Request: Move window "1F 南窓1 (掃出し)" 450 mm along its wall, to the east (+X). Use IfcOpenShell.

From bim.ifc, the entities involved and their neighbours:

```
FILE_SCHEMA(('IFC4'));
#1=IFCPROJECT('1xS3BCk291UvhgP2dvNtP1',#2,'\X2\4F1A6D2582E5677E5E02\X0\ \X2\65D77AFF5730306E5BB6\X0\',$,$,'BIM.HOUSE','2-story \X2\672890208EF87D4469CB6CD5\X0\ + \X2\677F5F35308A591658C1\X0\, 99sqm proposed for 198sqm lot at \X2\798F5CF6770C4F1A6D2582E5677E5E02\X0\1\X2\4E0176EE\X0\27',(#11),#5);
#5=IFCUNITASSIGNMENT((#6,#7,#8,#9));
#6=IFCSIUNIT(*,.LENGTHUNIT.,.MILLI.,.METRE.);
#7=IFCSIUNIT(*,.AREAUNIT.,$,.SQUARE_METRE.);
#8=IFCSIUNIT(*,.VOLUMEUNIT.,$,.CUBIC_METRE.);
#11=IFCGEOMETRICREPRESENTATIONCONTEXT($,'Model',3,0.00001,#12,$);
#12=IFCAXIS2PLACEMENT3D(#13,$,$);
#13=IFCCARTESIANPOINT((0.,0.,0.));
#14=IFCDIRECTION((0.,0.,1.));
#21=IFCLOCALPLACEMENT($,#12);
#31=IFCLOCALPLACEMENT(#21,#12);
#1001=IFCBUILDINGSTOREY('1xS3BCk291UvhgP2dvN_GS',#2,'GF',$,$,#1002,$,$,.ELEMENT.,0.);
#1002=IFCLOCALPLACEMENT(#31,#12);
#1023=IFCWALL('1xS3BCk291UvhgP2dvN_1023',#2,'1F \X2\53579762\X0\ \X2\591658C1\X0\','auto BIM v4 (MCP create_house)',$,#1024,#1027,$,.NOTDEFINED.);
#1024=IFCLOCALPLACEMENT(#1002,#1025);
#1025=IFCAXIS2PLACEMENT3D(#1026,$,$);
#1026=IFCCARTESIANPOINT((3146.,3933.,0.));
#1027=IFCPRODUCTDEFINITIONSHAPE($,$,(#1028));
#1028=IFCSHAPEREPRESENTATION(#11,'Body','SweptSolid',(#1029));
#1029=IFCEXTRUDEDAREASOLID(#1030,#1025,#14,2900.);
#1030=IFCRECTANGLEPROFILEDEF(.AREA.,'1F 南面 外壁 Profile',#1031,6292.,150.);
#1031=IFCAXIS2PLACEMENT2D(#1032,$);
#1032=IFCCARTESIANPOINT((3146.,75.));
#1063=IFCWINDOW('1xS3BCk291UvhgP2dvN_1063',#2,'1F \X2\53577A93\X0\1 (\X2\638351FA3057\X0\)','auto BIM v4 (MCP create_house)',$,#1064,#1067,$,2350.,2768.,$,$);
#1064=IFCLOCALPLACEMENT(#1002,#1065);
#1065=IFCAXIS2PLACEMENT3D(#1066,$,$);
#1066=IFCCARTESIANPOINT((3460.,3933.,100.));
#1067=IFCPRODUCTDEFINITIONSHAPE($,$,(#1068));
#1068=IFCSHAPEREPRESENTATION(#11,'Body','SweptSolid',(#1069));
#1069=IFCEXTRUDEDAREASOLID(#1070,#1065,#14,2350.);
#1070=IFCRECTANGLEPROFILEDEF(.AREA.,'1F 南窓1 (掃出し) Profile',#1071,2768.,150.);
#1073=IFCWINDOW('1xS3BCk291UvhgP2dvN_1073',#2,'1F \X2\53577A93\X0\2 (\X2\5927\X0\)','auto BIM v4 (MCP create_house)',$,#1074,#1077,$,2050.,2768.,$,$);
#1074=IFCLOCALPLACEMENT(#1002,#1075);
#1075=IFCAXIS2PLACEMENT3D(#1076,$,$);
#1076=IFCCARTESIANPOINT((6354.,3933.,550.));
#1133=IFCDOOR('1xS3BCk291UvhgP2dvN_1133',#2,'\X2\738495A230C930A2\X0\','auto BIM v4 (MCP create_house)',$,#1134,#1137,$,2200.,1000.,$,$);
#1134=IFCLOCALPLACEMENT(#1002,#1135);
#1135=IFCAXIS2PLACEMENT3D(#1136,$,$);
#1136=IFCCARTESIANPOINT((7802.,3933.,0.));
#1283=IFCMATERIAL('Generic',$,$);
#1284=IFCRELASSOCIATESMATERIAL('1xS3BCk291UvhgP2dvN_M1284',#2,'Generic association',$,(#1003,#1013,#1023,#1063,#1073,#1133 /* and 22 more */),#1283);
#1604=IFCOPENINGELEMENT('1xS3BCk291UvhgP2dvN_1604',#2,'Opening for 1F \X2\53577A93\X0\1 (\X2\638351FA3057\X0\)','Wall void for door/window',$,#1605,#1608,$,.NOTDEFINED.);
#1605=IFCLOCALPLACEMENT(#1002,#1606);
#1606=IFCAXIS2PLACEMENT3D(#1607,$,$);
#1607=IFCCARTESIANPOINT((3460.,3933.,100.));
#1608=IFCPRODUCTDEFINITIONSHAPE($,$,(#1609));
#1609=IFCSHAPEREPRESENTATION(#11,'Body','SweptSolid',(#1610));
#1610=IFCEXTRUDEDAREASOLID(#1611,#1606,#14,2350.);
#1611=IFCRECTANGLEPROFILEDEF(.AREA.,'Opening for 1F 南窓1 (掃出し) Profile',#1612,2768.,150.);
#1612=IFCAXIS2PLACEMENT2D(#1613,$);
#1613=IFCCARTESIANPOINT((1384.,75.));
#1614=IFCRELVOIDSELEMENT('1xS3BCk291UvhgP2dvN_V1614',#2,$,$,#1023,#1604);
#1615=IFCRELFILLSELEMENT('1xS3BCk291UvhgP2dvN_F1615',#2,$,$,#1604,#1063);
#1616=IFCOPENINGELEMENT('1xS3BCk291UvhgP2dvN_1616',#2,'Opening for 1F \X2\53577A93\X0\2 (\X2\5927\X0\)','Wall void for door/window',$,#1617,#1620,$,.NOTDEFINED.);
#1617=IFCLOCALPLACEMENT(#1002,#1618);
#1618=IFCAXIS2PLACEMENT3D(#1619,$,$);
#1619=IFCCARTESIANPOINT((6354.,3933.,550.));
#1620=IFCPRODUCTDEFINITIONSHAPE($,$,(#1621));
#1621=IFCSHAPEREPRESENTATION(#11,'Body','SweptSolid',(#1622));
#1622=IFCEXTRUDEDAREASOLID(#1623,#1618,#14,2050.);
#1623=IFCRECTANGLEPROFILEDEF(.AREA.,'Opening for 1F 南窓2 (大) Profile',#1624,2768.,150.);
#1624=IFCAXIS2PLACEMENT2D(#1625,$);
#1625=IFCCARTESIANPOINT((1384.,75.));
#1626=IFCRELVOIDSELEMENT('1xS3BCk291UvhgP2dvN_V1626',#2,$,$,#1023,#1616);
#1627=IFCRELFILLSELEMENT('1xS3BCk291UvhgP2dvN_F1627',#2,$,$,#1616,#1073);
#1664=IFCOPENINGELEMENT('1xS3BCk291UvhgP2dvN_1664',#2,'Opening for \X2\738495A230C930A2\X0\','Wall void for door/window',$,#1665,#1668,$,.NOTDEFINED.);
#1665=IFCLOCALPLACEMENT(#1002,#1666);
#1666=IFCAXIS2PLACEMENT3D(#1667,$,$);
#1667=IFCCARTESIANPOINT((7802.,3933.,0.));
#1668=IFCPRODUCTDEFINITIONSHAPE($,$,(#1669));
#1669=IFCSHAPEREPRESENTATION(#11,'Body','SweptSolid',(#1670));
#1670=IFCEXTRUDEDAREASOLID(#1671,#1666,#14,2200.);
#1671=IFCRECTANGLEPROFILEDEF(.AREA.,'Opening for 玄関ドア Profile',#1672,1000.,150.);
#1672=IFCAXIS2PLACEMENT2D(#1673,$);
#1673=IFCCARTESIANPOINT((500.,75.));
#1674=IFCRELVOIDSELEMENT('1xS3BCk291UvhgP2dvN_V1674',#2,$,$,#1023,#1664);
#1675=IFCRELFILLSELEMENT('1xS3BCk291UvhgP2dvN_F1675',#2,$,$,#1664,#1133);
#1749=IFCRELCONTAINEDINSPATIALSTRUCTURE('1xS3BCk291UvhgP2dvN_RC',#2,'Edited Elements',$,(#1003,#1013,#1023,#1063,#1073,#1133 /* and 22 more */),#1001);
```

```python
import ifcopenshell
import ifcopenshell.api.geometry
import ifcopenshell.util.placement

model = ifcopenshell.open("bim.ifc")

window = model.by_guid("1xS3BCk291UvhgP2dvN_1063")
opening = window.FillsVoids[0].RelatingOpeningElement
wall = opening.VoidsElements[0].RelatingBuildingElement

wall_matrix = ifcopenshell.util.placement.get_local_placement(wall.ObjectPlacement)
shift = wall_matrix[:3, 0] * 450.0
before = ifcopenshell.util.placement.get_local_placement(window.ObjectPlacement)[:3, 3].copy()

# The window is not placed relative to its opening, so move both.
for product in (opening, window):
    matrix = ifcopenshell.util.placement.get_local_placement(product.ObjectPlacement)
    matrix[:3, 3] += shift
    ifcopenshell.api.geometry.edit_object_placement(model, product=product, matrix=matrix, is_si=False)

after = ifcopenshell.util.placement.get_local_placement(window.ObjectPlacement)[:3, 3]
print("window moved by", (after - before).round(3) + 0.0)

model.write("bim_updated.ifc")
```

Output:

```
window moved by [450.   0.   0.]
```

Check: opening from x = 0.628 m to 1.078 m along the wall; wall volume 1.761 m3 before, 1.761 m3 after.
